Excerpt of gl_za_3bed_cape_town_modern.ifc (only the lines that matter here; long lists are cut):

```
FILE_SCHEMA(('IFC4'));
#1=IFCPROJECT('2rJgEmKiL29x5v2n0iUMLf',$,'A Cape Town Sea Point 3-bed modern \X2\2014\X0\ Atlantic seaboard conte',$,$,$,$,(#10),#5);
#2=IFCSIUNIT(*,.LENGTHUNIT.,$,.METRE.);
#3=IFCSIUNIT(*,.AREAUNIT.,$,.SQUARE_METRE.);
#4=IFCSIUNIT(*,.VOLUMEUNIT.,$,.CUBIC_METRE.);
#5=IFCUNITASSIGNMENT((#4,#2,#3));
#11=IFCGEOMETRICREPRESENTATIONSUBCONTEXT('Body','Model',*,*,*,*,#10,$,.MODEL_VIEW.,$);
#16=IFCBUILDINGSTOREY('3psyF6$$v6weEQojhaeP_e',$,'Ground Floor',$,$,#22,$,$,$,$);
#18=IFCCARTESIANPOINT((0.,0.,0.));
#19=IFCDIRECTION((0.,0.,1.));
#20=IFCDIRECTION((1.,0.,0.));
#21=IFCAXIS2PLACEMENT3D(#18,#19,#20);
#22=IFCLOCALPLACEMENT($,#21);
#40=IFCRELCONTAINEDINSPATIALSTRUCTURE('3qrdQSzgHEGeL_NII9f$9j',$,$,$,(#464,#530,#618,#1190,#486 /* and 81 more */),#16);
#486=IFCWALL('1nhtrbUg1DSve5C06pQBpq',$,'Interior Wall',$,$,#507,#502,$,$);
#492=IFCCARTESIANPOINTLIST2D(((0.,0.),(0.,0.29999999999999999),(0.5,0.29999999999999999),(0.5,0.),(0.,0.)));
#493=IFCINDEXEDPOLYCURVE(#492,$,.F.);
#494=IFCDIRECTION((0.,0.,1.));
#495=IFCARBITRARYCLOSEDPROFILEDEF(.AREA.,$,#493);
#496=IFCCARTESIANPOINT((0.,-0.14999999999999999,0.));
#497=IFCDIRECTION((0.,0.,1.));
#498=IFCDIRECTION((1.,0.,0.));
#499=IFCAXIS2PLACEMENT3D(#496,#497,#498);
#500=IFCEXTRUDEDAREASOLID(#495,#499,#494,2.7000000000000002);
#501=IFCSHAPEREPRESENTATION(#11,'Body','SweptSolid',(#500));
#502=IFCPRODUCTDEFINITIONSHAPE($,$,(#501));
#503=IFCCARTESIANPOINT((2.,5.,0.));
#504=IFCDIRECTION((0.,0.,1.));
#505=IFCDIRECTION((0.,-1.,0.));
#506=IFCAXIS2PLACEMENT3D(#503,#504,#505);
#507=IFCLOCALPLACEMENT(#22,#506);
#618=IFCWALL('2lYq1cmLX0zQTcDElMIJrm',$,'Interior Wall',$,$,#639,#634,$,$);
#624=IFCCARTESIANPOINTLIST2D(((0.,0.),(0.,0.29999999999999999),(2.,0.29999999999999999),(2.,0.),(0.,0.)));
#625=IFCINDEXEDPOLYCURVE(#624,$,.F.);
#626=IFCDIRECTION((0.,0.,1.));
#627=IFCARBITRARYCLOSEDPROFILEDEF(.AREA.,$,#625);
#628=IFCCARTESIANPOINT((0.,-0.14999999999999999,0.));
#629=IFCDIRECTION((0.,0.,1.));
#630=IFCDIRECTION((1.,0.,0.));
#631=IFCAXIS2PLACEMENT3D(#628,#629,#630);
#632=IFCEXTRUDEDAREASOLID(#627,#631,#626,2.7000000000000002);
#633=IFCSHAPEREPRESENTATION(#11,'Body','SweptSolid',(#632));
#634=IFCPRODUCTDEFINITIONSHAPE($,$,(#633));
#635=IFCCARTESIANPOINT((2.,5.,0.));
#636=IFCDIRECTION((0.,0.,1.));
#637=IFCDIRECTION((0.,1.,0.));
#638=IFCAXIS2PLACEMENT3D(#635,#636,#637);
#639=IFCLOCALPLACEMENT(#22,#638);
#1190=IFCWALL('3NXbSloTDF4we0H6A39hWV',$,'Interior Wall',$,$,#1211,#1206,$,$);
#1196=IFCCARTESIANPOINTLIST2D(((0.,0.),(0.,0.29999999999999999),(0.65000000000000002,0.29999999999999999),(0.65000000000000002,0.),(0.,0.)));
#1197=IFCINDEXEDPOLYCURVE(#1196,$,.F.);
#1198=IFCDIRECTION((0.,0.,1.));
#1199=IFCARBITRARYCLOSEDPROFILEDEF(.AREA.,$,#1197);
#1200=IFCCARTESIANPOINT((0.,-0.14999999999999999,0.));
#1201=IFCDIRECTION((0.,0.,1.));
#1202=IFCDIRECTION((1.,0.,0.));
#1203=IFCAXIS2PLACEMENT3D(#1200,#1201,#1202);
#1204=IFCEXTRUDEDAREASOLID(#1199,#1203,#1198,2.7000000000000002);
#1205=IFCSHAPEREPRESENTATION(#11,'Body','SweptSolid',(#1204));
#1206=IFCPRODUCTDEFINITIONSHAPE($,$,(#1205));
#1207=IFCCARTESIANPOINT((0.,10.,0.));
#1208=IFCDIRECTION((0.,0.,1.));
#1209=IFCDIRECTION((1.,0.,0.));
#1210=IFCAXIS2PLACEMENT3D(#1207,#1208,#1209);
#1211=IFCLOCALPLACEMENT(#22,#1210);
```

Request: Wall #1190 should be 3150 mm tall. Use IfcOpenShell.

```python
import ifcopenshell
import ifcopenshell.geom
import ifcopenshell.util.representation
import ifcopenshell.util.shape

model = ifcopenshell.open("gl_za_3bed_cape_town_modern.ifc")
settings = ifcopenshell.geom.settings()


def volume(element):
    """Net volume in cubic metres, openings subtracted."""
    shape = ifcopenshell.geom.create_shape(settings, element)
    return ifcopenshell.util.shape.get_volume(shape.geometry)


wall = model.by_guid("3NXbSloTDF4we0H6A39hWV")
before = volume(wall)

body = ifcopenshell.util.representation.get_representation(wall, "Model", "Body")
solid = body.Items[0]
old_height = solid.Depth
solid.Depth = 3.15
after = volume(wall)

print(f"height {old_height:g} -> {solid.Depth:g}, volume {before:.3f} -> {after:.3f} m3")

model.write("gl_za_3bed_cape_town_modern-out.ifc")
```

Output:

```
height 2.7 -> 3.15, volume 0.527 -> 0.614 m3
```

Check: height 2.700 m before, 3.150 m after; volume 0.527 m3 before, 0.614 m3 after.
